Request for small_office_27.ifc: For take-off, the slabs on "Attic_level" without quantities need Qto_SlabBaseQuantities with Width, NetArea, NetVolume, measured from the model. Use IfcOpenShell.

First a look at what the model holds.

```python
import ifcopenshell
import ifcopenshell.util.element
import ifcopenshell.util.unit

model = ifcopenshell.open("small_office_27.ifc")
print(model.schema)
for unit_type in ("LENGTHUNIT", "AREAUNIT", "VOLUMEUNIT"):
    print(unit_type, ifcopenshell.util.unit.calculate_unit_scale(model, unit_type))
storey = next(s for s in model.by_type("IfcBuildingStorey") if s.Name == "Attic_level")
slabs = [e for e in ifcopenshell.util.element.get_decomposition(storey) if e.is_a("IfcSlab")]
for e in sorted(slabs, key=lambda e: e.id()):
    print(e.id(), e.is_a(), e.Name, list(ifcopenshell.util.element.get_psets(e, qtos_only=True)), sep=" | ")
```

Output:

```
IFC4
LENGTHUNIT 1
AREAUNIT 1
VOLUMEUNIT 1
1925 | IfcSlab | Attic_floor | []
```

```python
import ifcopenshell
import ifcopenshell.api.pset
import ifcopenshell.geom
import ifcopenshell.util.element
import ifcopenshell.util.shape
import ifcopenshell.util.unit

model = ifcopenshell.open("small_office_27.ifc")
unit_scale = ifcopenshell.util.unit.calculate_unit_scale(model)
area_scale = ifcopenshell.util.unit.calculate_unit_scale(model, "AREAUNIT")
volume_scale = ifcopenshell.util.unit.calculate_unit_scale(model, "VOLUMEUNIT")
settings = ifcopenshell.geom.settings()

storey = next(s for s in model.by_type("IfcBuildingStorey") if s.Name == "Attic_level")
slabs = [e for e in ifcopenshell.util.element.get_decomposition(storey) if e.is_a("IfcSlab")]

for e in sorted(slabs, key=lambda e: e.id()):
    if ifcopenshell.util.element.get_psets(e, qtos_only=True, should_inherit=False):
        continue
    # Geometry comes back in metres, in the element's own axes.
    shape = ifcopenshell.geom.create_shape(settings, e)
    values = {
        "Width": ifcopenshell.util.shape.get_z(shape.geometry) / unit_scale,
        "NetArea": ifcopenshell.util.shape.get_footprint_area(shape.geometry) / area_scale,
        "NetVolume": ifcopenshell.util.shape.get_volume(shape.geometry) / volume_scale,
    }
    qto = ifcopenshell.api.pset.add_qto(model, product=e, name="Qto_SlabBaseQuantities")
    ifcopenshell.api.pset.edit_qto(model, qto=qto, properties=values)
    print(e.id(), {k: round(v, 3) for k, v in values.items()})

model.write("small_office_27_v2.ifc")
```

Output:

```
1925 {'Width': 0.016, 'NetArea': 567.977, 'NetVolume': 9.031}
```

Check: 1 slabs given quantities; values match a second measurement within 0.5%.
